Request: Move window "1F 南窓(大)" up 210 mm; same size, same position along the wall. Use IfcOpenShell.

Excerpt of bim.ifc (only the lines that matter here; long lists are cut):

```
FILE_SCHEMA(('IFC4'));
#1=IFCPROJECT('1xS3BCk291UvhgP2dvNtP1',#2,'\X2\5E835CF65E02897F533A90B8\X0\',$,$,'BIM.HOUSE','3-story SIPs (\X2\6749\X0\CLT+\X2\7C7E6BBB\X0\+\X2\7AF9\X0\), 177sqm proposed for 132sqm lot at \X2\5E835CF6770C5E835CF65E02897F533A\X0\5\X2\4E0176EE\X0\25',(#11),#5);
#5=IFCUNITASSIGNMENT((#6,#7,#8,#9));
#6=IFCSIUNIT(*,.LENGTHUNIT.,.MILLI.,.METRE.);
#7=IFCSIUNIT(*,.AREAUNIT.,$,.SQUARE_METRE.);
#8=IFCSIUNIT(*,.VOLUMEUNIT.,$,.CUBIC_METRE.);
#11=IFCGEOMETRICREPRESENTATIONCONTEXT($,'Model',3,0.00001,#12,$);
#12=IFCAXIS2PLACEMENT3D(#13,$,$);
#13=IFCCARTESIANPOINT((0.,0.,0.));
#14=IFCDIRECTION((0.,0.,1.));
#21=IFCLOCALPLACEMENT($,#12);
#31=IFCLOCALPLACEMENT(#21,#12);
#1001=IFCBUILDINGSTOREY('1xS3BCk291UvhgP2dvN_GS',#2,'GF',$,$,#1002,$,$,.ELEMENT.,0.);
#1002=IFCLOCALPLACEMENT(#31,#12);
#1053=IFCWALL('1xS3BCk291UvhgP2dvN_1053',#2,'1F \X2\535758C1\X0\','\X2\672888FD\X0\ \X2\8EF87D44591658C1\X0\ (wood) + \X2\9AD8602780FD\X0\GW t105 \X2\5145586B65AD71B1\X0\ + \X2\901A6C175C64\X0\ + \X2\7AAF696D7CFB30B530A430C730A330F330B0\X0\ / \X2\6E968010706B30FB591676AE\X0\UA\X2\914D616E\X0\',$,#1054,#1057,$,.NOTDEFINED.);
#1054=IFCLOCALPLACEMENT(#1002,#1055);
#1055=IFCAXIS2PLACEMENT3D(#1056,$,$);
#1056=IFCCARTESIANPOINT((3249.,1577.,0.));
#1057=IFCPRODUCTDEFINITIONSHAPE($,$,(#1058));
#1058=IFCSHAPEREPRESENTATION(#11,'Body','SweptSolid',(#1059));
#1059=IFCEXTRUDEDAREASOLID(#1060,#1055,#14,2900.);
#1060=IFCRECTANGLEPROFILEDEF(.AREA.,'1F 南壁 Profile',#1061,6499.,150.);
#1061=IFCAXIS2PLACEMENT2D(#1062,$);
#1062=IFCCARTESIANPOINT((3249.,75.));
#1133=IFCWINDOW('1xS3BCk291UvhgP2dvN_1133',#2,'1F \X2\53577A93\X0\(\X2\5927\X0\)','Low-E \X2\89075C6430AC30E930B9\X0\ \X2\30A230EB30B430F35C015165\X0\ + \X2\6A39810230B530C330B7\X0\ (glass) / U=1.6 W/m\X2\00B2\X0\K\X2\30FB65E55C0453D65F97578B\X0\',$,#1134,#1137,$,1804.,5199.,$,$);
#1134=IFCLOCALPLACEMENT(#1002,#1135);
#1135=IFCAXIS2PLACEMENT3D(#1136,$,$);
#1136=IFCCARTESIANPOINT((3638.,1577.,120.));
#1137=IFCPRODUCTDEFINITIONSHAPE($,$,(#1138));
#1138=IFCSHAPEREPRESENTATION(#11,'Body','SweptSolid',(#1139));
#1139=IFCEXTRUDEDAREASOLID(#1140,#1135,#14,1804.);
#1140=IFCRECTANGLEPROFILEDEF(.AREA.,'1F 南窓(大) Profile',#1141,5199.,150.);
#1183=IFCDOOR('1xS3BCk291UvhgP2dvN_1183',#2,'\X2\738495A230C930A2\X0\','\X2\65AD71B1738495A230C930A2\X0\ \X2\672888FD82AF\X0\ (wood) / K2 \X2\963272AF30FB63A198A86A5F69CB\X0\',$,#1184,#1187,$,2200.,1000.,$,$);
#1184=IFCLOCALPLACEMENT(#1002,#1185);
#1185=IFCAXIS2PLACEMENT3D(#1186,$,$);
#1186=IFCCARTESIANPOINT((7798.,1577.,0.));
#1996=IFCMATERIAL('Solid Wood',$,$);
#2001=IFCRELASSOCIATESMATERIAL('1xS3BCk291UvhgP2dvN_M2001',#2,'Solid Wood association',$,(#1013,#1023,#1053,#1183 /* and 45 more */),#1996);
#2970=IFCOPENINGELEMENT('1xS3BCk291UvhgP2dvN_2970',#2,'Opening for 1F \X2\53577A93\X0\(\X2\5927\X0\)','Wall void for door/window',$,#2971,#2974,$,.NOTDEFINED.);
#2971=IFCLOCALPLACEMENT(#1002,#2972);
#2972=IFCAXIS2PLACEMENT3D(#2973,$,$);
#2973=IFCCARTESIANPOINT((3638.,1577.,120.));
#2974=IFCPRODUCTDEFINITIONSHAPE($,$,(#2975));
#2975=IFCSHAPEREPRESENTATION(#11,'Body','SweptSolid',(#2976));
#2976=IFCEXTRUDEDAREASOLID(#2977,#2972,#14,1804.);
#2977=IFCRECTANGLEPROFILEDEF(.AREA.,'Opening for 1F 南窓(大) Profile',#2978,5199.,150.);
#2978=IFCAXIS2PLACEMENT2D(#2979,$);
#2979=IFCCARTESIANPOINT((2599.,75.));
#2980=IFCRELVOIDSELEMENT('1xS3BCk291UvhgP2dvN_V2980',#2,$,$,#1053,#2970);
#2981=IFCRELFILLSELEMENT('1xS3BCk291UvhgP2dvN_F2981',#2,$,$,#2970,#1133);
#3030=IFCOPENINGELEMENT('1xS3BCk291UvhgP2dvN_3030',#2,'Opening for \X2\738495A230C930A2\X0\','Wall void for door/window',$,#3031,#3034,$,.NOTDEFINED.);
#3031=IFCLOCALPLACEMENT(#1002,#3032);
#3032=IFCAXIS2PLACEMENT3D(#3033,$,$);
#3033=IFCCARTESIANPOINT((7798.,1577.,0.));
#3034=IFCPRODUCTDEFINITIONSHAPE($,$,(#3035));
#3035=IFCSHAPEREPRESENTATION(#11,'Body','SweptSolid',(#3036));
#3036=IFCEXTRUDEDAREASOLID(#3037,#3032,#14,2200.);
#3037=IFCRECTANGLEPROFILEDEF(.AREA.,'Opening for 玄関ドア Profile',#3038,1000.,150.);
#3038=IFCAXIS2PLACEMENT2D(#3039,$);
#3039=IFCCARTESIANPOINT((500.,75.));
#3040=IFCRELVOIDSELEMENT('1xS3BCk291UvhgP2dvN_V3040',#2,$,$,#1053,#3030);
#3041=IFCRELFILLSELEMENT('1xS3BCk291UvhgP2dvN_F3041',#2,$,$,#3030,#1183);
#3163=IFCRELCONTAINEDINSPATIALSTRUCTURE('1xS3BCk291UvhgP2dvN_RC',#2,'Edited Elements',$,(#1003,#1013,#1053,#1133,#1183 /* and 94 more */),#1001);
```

```python
import numpy as np
import ifcopenshell
import ifcopenshell.api.geometry
import ifcopenshell.util.placement
import ifcopenshell.util.unit

model = ifcopenshell.open("bim.ifc")
unit_scale = ifcopenshell.util.unit.calculate_unit_scale(model)

window = model.by_guid("1xS3BCk291UvhgP2dvN_1133")
opening = window.FillsVoids[0].RelatingOpeningElement
dz = 0.21 / unit_scale

shift = np.array([0.0, 0.0, dz])
# The window is not placed relative to its opening, so move both.
for product in (opening, window):
    matrix = ifcopenshell.util.placement.get_local_placement(product.ObjectPlacement)
    matrix[:3, 3] += shift
    ifcopenshell.api.geometry.edit_object_placement(model, product=product, matrix=matrix, is_si=False)

print(f"moved by {dz * unit_scale:+.3f} m")

model.write("bim_v2.ifc")
```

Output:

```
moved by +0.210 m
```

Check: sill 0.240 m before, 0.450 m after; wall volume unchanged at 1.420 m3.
